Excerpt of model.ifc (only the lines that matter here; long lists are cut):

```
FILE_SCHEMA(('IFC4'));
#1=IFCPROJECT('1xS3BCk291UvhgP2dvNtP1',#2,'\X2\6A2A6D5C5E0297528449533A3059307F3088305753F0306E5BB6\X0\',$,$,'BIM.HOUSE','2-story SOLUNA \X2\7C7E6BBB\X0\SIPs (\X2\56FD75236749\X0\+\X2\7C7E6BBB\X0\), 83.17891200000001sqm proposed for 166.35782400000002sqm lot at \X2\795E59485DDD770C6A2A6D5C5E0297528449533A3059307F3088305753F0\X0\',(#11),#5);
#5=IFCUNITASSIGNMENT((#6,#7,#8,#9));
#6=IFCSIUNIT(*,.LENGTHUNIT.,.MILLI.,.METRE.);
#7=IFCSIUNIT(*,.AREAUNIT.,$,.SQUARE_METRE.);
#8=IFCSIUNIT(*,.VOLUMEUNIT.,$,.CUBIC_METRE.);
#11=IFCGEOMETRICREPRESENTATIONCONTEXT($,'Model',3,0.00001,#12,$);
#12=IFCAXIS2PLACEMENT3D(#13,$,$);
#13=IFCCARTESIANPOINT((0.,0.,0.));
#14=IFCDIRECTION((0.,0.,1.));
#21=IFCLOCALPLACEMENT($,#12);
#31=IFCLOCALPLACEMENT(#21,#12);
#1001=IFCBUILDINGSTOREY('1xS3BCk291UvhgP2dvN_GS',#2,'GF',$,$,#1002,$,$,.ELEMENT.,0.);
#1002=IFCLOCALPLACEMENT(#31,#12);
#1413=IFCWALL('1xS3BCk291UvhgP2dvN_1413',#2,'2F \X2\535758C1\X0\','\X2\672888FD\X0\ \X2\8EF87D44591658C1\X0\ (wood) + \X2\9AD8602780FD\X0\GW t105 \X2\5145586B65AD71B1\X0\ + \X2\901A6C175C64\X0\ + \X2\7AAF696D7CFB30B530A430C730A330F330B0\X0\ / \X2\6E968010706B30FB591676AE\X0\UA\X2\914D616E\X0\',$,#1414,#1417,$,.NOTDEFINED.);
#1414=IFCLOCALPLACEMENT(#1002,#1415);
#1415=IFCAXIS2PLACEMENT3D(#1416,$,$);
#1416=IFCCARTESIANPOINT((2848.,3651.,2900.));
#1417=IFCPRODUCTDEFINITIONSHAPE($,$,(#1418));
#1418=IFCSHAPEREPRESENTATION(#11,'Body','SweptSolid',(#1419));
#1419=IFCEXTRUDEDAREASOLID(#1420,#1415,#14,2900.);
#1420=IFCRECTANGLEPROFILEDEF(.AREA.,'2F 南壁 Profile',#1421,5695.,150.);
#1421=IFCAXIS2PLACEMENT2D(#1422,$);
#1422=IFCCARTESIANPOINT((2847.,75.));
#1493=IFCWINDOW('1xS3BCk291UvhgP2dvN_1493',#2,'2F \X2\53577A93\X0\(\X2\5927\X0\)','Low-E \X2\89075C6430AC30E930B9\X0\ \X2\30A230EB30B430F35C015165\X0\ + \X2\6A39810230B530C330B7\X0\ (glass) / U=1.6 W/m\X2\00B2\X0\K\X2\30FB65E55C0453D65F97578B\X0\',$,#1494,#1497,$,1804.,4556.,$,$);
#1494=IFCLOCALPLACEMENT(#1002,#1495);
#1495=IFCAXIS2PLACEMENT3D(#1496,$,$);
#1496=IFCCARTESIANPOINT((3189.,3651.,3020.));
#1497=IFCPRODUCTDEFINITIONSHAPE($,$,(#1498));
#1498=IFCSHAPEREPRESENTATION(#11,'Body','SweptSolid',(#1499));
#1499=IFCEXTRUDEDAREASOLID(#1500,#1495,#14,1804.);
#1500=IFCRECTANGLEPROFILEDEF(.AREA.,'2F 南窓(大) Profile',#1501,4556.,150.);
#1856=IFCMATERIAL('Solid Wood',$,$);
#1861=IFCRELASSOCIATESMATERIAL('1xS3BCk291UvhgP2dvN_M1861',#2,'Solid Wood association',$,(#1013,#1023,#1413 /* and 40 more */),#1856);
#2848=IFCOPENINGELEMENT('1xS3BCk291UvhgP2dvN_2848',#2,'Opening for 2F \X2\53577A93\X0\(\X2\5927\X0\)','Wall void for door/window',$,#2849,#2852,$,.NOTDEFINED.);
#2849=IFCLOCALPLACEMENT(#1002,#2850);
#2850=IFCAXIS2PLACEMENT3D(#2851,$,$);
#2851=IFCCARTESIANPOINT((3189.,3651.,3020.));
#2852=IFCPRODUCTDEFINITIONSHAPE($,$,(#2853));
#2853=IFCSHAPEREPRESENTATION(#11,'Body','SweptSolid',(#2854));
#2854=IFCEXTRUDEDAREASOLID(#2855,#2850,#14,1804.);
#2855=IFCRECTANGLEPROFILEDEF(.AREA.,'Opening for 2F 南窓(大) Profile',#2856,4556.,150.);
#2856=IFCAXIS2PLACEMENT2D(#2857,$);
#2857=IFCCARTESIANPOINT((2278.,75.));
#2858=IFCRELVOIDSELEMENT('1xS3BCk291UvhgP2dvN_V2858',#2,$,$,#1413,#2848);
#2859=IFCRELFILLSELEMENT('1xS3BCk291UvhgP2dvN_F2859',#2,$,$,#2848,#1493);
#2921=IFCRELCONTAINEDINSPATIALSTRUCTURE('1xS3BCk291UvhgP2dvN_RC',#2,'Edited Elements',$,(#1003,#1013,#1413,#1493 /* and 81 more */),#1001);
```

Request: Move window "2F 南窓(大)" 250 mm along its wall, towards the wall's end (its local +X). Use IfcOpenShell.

```python
import ifcopenshell
import ifcopenshell.api.geometry
import ifcopenshell.util.placement

model = ifcopenshell.open("model.ifc")

window = model.by_guid("1xS3BCk291UvhgP2dvN_1493")
opening = window.FillsVoids[0].RelatingOpeningElement
wall = opening.VoidsElements[0].RelatingBuildingElement

wall_matrix = ifcopenshell.util.placement.get_local_placement(wall.ObjectPlacement)
shift = wall_matrix[:3, 0] * 250.0
before = ifcopenshell.util.placement.get_local_placement(window.ObjectPlacement)[:3, 3].copy()

# The window is not placed relative to its opening, so move both.
for product in (opening, window):
    matrix = ifcopenshell.util.placement.get_local_placement(product.ObjectPlacement)
    matrix[:3, 3] += shift
    ifcopenshell.api.geometry.edit_object_placement(model, product=product, matrix=matrix, is_si=False)

after = ifcopenshell.util.placement.get_local_placement(window.ObjectPlacement)[:3, 3]
print("window moved by", (after - before).round(3) + 0.0)

model.write("model_rev.ifc")
```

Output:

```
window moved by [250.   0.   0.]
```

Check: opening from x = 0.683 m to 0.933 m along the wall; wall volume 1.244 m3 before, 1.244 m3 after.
